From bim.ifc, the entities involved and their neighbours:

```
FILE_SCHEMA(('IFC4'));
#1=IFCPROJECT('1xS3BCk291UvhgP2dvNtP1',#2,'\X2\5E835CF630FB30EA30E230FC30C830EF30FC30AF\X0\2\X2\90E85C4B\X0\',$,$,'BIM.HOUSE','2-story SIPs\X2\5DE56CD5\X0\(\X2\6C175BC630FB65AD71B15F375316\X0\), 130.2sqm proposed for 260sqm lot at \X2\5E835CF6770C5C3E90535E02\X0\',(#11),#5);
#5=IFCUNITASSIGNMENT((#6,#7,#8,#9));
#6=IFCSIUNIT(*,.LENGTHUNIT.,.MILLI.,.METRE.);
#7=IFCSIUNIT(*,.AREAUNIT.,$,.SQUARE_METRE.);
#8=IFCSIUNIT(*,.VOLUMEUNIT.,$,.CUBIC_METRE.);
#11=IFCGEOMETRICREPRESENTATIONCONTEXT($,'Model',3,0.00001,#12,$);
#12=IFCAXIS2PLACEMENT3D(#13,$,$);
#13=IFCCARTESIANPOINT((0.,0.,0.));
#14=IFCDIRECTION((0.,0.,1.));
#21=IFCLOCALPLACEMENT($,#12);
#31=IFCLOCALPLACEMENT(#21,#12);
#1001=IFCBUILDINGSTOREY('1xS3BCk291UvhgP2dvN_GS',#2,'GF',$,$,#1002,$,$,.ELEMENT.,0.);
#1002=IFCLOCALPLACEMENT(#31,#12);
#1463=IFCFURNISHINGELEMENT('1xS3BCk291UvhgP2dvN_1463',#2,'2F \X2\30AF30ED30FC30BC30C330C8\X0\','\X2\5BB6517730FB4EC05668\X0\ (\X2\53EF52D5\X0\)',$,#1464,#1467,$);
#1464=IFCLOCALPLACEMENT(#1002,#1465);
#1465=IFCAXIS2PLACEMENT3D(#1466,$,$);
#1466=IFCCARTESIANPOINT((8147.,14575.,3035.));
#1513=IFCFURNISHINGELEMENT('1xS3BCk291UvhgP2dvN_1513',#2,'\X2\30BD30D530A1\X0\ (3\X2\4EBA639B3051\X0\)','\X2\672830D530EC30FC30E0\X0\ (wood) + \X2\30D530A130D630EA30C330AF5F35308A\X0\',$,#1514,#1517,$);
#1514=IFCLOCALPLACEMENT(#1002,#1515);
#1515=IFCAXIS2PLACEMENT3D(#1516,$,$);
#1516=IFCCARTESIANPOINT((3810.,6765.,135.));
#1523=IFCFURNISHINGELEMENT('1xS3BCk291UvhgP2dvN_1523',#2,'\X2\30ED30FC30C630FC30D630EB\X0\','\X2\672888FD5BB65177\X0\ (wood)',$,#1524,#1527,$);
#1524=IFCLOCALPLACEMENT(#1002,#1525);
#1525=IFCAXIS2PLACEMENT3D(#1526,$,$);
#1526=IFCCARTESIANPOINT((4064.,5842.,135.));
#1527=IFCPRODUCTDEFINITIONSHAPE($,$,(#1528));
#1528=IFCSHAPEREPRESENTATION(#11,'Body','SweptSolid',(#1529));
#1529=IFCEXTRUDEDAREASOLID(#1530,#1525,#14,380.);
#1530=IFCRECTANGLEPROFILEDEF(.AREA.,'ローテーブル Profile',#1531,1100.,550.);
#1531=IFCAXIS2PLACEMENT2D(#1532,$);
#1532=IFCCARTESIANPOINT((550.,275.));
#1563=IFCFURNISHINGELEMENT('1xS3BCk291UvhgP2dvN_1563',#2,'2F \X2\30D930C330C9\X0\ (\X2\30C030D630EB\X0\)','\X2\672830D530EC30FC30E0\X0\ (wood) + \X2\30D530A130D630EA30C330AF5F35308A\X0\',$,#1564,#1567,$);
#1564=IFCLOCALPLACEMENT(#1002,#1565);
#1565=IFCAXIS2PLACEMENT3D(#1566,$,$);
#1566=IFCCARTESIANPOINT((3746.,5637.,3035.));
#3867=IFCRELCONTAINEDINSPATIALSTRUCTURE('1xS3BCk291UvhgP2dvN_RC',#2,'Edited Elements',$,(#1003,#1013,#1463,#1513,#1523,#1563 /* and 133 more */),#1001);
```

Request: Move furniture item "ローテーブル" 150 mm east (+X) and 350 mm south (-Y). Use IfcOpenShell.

```python
import ifcopenshell
import ifcopenshell.api.geometry
import ifcopenshell.util.placement
import ifcopenshell.util.unit

model = ifcopenshell.open("bim.ifc")
unit_scale = ifcopenshell.util.unit.calculate_unit_scale(model)

item = model.by_id(1523)
matrix = ifcopenshell.util.placement.get_local_placement(item.ObjectPlacement)
matrix[0, 3] += 0.15 / unit_scale
matrix[1, 3] -= 0.35 / unit_scale
ifcopenshell.api.geometry.edit_object_placement(model, product=item, matrix=matrix, is_si=False)

print(ifcopenshell.util.placement.get_local_placement(item.ObjectPlacement).round(3) + 0.0)

model.write("bim_edited.ifc")
```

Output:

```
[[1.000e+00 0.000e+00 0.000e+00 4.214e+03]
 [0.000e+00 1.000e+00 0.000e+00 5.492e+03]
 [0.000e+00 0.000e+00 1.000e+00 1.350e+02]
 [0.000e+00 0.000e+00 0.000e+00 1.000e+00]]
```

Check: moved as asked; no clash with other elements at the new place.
